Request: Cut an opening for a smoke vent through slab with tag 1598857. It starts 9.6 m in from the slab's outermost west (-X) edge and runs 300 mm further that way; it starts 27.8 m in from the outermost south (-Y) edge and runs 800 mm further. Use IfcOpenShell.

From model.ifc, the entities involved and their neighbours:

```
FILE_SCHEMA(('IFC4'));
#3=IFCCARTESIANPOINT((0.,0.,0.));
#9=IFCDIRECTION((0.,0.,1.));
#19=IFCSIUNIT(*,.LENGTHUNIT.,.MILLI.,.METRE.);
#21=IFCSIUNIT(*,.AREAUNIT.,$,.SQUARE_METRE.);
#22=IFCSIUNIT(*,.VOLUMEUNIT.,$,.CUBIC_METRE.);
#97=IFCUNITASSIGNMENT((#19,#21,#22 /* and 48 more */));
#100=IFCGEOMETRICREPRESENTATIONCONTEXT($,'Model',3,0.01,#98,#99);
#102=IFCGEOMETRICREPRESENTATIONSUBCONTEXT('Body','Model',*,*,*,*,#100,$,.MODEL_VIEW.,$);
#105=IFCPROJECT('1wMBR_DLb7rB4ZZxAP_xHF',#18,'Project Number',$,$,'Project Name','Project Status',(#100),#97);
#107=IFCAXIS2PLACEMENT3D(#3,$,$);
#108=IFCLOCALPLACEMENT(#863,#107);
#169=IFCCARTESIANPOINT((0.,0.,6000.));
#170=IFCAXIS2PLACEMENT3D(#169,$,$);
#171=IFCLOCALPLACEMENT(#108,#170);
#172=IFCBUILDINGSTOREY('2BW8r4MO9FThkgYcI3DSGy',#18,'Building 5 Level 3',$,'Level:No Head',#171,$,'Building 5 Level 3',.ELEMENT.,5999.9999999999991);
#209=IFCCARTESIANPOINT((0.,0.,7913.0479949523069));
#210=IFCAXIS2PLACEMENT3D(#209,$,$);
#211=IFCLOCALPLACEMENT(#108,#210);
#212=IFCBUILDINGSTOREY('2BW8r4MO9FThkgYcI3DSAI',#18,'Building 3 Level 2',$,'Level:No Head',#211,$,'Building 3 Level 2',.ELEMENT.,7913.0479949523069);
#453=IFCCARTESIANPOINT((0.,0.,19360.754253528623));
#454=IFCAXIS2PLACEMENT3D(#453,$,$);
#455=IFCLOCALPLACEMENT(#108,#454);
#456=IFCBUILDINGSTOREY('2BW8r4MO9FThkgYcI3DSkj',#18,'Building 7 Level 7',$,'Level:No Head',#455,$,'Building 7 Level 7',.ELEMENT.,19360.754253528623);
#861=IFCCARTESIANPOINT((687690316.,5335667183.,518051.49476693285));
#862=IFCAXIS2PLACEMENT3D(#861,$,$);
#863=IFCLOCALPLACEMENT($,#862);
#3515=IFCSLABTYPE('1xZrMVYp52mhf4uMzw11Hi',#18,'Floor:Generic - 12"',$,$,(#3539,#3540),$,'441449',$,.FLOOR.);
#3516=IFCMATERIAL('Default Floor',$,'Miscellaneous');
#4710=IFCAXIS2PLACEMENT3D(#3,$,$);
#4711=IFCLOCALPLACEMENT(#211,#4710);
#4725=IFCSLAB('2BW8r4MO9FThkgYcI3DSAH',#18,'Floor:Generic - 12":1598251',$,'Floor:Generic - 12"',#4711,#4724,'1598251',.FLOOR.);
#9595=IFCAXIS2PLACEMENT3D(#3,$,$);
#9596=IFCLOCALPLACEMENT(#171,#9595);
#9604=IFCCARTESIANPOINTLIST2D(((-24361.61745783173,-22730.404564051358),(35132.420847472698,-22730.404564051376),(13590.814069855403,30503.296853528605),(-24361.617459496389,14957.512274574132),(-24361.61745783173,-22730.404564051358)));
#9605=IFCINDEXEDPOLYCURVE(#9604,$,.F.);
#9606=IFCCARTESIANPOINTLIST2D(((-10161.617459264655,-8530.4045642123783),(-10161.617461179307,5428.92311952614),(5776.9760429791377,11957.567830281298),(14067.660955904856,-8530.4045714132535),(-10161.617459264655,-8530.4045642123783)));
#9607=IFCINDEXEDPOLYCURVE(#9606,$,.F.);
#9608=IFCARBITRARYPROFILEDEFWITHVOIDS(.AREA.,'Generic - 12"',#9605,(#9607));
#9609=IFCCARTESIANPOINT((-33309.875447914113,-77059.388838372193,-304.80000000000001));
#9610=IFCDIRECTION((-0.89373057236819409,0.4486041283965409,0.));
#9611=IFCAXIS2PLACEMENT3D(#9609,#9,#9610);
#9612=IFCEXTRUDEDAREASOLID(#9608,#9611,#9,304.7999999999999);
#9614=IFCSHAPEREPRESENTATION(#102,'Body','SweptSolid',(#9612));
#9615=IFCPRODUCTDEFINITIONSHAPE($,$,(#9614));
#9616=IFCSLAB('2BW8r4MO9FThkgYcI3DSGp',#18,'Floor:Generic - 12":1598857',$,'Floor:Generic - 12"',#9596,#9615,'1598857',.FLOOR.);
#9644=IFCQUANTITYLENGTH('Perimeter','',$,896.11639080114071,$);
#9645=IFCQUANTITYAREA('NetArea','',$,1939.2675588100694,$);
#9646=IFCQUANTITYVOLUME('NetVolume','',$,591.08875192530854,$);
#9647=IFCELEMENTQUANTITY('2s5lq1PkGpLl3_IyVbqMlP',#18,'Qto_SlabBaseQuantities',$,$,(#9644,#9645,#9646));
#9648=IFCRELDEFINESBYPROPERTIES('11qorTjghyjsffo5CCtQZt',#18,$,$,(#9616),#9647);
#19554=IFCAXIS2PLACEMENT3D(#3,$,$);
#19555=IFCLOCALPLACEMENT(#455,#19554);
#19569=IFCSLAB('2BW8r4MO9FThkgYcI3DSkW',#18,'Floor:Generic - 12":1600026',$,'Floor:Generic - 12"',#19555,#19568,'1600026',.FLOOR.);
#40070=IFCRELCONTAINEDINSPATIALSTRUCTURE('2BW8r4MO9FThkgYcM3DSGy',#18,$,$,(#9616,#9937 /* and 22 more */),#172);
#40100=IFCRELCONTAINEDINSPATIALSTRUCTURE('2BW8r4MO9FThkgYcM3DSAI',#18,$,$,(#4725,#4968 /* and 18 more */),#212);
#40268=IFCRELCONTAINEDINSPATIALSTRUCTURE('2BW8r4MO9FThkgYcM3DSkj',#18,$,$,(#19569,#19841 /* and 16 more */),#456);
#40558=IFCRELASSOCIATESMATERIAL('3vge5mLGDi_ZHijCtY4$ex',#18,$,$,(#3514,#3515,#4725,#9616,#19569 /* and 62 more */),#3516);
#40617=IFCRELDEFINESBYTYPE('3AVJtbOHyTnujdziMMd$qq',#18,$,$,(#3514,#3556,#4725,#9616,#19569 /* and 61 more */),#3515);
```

```python
import numpy as np
import ifcopenshell
import ifcopenshell.api.feature
import ifcopenshell.api.geometry
import ifcopenshell.api.pset
import ifcopenshell.api.root
import ifcopenshell.geom
import ifcopenshell.util.element
import ifcopenshell.util.placement
import ifcopenshell.util.representation
import ifcopenshell.util.shape
import ifcopenshell.util.unit

model = ifcopenshell.open("model.ifc")
unit_scale = ifcopenshell.util.unit.calculate_unit_scale(model)
area_scale = ifcopenshell.util.unit.calculate_unit_scale(model, "AREAUNIT")
volume_scale = ifcopenshell.util.unit.calculate_unit_scale(model, "VOLUMEUNIT")
settings = ifcopenshell.geom.settings()


def volume(element):
    """Net volume in cubic metres, openings subtracted."""
    shape = ifcopenshell.geom.create_shape(settings, element)
    return ifcopenshell.util.shape.get_volume(shape.geometry)


slab = model.by_id(9616)
before = volume(slab)

# Extent in the slab's own axes, in metres. The edges named are its -X and -Y sides.
slab_shape = ifcopenshell.geom.create_shape(settings, slab)
vertices = ifcopenshell.util.shape.get_vertices(slab_shape.geometry)
x_min, y_min, bottom = vertices.min(axis=0)
top = vertices[:, 2].max()

opening = ifcopenshell.api.root.create_entity(model, ifc_class="IfcOpeningElement", name="Smoke vent opening", predefined_type="OPENING")
context = ifcopenshell.util.representation.get_context(model, "Model", "Body", "MODEL_VIEW")
width, depth = 0.3, 0.8
outline = [(0.0, 0.0), (width, 0.0), (width, depth), (0.0, depth), (0.0, 0.0)]
# Overshoot both faces by 50 mm so the cut is clean.
shape = ifcopenshell.api.geometry.add_slab_representation(
    model, context=context, depth=top - bottom + 0.1, polyline=outline
)
ifcopenshell.api.geometry.assign_representation(model, product=opening, representation=shape)

matrix = ifcopenshell.util.placement.get_local_placement(slab.ObjectPlacement)
matrix[:, 3] = matrix @ np.append(np.array([x_min + 9.6, y_min + 27.8, bottom - 0.05]) / unit_scale, 1.0)
ifcopenshell.api.geometry.edit_object_placement(model, product=opening, matrix=matrix, is_si=False)
ifcopenshell.api.feature.add_feature(model, feature=opening, element=slab)

after = volume(slab)

# Update the slab's stored quantities.
qto = model.by_id(ifcopenshell.util.element.get_pset(slab, "Qto_SlabBaseQuantities", should_inherit=False)["id"])
ifcopenshell.api.pset.edit_qto(model, qto=qto, properties={
    "NetArea": after / (top - bottom) / area_scale,
    "NetVolume": after / volume_scale,
})

print(f"slab volume {before:.3f} -> {after:.3f} m3")

model.write("model_edited.ifc")
```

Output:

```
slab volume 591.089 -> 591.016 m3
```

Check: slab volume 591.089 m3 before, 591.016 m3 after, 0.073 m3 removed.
